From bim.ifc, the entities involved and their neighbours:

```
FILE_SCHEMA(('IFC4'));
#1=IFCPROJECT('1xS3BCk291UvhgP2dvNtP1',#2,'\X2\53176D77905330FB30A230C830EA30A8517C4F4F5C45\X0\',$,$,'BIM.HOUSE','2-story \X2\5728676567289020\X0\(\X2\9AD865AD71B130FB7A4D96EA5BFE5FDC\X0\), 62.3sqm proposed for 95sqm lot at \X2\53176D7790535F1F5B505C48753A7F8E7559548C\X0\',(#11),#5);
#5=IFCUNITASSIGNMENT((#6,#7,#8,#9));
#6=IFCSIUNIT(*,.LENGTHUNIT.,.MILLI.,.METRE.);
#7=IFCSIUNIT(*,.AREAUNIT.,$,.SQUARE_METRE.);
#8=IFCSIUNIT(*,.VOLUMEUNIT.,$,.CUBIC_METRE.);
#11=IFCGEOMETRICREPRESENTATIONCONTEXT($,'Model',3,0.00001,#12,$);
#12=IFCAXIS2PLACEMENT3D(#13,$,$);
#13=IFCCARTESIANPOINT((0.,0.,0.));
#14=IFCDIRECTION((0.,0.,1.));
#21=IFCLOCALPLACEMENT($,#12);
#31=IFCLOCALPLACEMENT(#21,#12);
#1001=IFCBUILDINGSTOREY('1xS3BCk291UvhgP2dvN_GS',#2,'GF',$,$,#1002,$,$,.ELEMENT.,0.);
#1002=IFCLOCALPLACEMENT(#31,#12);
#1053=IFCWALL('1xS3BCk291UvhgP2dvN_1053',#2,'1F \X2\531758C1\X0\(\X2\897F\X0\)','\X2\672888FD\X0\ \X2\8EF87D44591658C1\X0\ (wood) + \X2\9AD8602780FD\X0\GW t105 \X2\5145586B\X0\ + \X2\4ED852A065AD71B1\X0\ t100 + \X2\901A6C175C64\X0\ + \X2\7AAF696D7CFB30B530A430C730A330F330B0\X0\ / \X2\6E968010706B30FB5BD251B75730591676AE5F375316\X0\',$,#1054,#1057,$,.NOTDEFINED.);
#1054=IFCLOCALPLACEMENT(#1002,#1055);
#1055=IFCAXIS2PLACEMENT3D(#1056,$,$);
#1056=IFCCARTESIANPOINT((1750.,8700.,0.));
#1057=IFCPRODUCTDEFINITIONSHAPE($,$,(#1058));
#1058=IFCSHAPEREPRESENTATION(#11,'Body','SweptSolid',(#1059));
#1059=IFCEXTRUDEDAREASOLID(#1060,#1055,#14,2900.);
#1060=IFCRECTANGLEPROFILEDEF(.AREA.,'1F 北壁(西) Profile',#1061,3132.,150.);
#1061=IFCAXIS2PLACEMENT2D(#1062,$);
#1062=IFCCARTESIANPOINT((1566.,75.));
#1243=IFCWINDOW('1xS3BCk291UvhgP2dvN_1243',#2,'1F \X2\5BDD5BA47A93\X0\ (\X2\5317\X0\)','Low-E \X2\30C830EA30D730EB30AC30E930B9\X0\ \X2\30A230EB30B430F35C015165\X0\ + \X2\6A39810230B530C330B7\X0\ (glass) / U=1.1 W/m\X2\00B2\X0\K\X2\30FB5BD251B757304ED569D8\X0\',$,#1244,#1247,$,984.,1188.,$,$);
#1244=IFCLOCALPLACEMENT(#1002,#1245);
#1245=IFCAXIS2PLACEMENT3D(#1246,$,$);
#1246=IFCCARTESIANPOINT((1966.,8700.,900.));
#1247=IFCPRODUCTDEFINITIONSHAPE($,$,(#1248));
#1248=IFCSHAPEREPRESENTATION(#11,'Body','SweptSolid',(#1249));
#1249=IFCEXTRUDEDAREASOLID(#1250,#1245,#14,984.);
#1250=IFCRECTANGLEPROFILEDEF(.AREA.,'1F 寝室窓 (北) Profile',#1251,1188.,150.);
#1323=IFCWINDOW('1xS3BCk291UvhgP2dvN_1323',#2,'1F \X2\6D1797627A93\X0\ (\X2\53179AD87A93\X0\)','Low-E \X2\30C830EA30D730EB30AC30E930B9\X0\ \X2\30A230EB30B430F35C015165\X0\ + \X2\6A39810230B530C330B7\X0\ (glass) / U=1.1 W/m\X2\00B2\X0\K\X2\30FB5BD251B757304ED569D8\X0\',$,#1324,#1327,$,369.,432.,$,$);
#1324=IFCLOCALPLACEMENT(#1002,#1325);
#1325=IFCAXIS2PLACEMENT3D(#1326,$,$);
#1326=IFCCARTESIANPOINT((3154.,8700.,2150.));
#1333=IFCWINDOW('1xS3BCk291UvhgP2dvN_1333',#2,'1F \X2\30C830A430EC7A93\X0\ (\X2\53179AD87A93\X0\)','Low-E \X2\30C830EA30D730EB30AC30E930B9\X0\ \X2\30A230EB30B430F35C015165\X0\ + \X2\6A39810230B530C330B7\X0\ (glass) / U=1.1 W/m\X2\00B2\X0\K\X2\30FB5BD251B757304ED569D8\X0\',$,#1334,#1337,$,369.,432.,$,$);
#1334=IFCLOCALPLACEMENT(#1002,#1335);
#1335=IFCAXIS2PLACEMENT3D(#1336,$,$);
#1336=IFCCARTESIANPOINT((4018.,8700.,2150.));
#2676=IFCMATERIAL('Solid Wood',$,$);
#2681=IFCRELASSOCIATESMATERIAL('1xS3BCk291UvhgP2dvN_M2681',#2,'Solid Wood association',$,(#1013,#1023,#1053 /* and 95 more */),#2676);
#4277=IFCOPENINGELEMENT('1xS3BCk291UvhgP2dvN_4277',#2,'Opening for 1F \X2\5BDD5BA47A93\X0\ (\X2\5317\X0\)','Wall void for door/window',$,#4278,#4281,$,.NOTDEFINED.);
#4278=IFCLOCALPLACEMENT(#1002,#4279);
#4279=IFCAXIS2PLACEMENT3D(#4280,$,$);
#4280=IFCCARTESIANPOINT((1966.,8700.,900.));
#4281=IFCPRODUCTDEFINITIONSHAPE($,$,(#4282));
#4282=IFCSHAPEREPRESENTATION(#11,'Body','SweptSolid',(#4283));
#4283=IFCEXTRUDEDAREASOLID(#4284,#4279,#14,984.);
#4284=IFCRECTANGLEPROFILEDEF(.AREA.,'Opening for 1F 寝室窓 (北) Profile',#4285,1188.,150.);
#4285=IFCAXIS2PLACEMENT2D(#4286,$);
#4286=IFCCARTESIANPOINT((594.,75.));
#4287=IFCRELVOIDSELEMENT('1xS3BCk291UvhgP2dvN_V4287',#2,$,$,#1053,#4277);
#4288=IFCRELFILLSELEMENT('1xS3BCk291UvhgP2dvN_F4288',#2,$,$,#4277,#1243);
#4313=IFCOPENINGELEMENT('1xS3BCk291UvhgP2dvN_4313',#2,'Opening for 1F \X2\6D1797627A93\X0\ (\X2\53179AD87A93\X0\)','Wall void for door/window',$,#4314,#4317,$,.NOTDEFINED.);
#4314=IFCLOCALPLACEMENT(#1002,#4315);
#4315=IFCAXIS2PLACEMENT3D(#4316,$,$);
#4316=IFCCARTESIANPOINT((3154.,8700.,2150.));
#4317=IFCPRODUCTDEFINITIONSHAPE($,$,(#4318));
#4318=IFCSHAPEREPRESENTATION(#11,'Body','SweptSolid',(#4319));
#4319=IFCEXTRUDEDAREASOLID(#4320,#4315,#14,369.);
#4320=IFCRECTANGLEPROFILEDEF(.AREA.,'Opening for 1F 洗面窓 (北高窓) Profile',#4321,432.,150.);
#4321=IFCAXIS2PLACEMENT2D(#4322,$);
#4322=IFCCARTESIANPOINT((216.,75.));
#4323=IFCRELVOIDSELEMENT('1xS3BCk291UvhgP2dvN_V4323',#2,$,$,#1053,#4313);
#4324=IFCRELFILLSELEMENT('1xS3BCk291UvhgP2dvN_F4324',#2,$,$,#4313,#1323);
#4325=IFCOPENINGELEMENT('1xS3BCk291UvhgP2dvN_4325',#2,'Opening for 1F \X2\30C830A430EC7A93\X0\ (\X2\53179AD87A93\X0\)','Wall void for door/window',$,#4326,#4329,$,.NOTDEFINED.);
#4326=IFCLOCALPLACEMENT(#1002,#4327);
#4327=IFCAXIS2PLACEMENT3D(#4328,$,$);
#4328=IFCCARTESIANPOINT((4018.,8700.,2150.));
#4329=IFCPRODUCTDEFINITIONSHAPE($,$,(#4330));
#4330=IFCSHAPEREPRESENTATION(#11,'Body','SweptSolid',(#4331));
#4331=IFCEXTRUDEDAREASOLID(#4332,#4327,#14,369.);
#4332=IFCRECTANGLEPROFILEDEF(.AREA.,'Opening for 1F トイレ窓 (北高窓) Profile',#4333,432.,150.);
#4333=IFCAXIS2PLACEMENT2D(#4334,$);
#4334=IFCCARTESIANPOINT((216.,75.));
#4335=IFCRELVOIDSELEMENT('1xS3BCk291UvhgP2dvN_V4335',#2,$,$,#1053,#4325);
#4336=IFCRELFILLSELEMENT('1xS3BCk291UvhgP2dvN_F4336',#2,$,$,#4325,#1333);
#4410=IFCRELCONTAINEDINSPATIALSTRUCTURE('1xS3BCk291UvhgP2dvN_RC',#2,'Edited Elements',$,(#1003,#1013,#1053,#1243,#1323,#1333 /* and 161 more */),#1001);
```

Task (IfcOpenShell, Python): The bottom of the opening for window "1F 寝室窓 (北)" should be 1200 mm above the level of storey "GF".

```python
import numpy as np
import ifcopenshell
import ifcopenshell.api.geometry
import ifcopenshell.geom
import ifcopenshell.util.element
import ifcopenshell.util.placement
import ifcopenshell.util.shape
import ifcopenshell.util.unit

model = ifcopenshell.open("bim.ifc")
unit_scale = ifcopenshell.util.unit.calculate_unit_scale(model)

window = model.by_guid("1xS3BCk291UvhgP2dvN_1243")
opening = window.FillsVoids[0].RelatingOpeningElement
storey = ifcopenshell.util.element.get_container(window, ifc_class="IfcBuildingStorey")
level = ifcopenshell.util.placement.get_local_placement(storey.ObjectPlacement)[2, 3]

# The opening's origin need not be at the sill, so measure its lowest point.
shape = ifcopenshell.geom.create_shape(ifcopenshell.geom.settings(), opening)
bottom = ifcopenshell.util.shape.get_shape_bottom_elevation(shape, shape.geometry) / unit_scale
dz = level + 1200.0 - bottom

shift = np.array([0.0, 0.0, dz])
# The window is not placed relative to its opening, so move both.
for product in (opening, window):
    matrix = ifcopenshell.util.placement.get_local_placement(product.ObjectPlacement)
    matrix[:3, 3] += shift
    ifcopenshell.api.geometry.edit_object_placement(model, product=product, matrix=matrix, is_si=False)

print(f"moved by {dz * unit_scale:+.3f} m")

model.write("bim_rev.ifc")
```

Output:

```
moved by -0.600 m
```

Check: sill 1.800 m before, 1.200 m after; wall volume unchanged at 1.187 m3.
